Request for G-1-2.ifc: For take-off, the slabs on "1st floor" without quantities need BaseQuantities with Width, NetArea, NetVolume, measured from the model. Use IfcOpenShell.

First a look at what the model holds.

```python
import ifcopenshell
import ifcopenshell.util.element
import ifcopenshell.util.unit

model = ifcopenshell.open("G-1-2.ifc")
print(model.schema)
for unit_type in ("LENGTHUNIT", "AREAUNIT", "VOLUMEUNIT"):
    print(unit_type, ifcopenshell.util.unit.calculate_unit_scale(model, unit_type))
storey = next(s for s in model.by_type("IfcBuildingStorey") if s.Name == "1st floor")
slabs = [e for e in ifcopenshell.util.element.get_decomposition(storey) if e.is_a("IfcSlab")]
for e in sorted(slabs, key=lambda e: e.id()):
    print(e.id(), e.is_a(), e.Name, list(ifcopenshell.util.element.get_psets(e, qtos_only=True)), sep=" | ")
```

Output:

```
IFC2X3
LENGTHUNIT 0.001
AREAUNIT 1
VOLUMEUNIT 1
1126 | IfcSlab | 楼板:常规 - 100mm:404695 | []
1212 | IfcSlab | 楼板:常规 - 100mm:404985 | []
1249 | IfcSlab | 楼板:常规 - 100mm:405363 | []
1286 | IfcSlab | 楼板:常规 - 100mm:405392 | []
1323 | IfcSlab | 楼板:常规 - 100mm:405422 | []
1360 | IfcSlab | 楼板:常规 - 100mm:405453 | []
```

```python
import ifcopenshell
import ifcopenshell.api.pset
import ifcopenshell.geom
import ifcopenshell.util.element
import ifcopenshell.util.shape
import ifcopenshell.util.unit

model = ifcopenshell.open("G-1-2.ifc")
unit_scale = ifcopenshell.util.unit.calculate_unit_scale(model)
area_scale = ifcopenshell.util.unit.calculate_unit_scale(model, "AREAUNIT")
volume_scale = ifcopenshell.util.unit.calculate_unit_scale(model, "VOLUMEUNIT")
settings = ifcopenshell.geom.settings()

storey = next(s for s in model.by_type("IfcBuildingStorey") if s.Name == "1st floor")
slabs = [e for e in ifcopenshell.util.element.get_decomposition(storey) if e.is_a("IfcSlab")]

for e in sorted(slabs, key=lambda e: e.id()):
    if ifcopenshell.util.element.get_psets(e, qtos_only=True, should_inherit=False):
        continue
    # Geometry comes back in metres, in the element's own axes.
    shape = ifcopenshell.geom.create_shape(settings, e)
    values = {
        "Width": ifcopenshell.util.shape.get_z(shape.geometry) / unit_scale,
        "NetArea": ifcopenshell.util.shape.get_footprint_area(shape.geometry) / area_scale,
        "NetVolume": ifcopenshell.util.shape.get_volume(shape.geometry) / volume_scale,
    }
    qto = ifcopenshell.api.pset.add_qto(model, product=e, name="BaseQuantities")
    ifcopenshell.api.pset.edit_qto(model, qto=qto, properties=values)
    print(e.id(), {k: round(v, 3) for k, v in values.items()})

model.write("G-1-2_v2.ifc")
```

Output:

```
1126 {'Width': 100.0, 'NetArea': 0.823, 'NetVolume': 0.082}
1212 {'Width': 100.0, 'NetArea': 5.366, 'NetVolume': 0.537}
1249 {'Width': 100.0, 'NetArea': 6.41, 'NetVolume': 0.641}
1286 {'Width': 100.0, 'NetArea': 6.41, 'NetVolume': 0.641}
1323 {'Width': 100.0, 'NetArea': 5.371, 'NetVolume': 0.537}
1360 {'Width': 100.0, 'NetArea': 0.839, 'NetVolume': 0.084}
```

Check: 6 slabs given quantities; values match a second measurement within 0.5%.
